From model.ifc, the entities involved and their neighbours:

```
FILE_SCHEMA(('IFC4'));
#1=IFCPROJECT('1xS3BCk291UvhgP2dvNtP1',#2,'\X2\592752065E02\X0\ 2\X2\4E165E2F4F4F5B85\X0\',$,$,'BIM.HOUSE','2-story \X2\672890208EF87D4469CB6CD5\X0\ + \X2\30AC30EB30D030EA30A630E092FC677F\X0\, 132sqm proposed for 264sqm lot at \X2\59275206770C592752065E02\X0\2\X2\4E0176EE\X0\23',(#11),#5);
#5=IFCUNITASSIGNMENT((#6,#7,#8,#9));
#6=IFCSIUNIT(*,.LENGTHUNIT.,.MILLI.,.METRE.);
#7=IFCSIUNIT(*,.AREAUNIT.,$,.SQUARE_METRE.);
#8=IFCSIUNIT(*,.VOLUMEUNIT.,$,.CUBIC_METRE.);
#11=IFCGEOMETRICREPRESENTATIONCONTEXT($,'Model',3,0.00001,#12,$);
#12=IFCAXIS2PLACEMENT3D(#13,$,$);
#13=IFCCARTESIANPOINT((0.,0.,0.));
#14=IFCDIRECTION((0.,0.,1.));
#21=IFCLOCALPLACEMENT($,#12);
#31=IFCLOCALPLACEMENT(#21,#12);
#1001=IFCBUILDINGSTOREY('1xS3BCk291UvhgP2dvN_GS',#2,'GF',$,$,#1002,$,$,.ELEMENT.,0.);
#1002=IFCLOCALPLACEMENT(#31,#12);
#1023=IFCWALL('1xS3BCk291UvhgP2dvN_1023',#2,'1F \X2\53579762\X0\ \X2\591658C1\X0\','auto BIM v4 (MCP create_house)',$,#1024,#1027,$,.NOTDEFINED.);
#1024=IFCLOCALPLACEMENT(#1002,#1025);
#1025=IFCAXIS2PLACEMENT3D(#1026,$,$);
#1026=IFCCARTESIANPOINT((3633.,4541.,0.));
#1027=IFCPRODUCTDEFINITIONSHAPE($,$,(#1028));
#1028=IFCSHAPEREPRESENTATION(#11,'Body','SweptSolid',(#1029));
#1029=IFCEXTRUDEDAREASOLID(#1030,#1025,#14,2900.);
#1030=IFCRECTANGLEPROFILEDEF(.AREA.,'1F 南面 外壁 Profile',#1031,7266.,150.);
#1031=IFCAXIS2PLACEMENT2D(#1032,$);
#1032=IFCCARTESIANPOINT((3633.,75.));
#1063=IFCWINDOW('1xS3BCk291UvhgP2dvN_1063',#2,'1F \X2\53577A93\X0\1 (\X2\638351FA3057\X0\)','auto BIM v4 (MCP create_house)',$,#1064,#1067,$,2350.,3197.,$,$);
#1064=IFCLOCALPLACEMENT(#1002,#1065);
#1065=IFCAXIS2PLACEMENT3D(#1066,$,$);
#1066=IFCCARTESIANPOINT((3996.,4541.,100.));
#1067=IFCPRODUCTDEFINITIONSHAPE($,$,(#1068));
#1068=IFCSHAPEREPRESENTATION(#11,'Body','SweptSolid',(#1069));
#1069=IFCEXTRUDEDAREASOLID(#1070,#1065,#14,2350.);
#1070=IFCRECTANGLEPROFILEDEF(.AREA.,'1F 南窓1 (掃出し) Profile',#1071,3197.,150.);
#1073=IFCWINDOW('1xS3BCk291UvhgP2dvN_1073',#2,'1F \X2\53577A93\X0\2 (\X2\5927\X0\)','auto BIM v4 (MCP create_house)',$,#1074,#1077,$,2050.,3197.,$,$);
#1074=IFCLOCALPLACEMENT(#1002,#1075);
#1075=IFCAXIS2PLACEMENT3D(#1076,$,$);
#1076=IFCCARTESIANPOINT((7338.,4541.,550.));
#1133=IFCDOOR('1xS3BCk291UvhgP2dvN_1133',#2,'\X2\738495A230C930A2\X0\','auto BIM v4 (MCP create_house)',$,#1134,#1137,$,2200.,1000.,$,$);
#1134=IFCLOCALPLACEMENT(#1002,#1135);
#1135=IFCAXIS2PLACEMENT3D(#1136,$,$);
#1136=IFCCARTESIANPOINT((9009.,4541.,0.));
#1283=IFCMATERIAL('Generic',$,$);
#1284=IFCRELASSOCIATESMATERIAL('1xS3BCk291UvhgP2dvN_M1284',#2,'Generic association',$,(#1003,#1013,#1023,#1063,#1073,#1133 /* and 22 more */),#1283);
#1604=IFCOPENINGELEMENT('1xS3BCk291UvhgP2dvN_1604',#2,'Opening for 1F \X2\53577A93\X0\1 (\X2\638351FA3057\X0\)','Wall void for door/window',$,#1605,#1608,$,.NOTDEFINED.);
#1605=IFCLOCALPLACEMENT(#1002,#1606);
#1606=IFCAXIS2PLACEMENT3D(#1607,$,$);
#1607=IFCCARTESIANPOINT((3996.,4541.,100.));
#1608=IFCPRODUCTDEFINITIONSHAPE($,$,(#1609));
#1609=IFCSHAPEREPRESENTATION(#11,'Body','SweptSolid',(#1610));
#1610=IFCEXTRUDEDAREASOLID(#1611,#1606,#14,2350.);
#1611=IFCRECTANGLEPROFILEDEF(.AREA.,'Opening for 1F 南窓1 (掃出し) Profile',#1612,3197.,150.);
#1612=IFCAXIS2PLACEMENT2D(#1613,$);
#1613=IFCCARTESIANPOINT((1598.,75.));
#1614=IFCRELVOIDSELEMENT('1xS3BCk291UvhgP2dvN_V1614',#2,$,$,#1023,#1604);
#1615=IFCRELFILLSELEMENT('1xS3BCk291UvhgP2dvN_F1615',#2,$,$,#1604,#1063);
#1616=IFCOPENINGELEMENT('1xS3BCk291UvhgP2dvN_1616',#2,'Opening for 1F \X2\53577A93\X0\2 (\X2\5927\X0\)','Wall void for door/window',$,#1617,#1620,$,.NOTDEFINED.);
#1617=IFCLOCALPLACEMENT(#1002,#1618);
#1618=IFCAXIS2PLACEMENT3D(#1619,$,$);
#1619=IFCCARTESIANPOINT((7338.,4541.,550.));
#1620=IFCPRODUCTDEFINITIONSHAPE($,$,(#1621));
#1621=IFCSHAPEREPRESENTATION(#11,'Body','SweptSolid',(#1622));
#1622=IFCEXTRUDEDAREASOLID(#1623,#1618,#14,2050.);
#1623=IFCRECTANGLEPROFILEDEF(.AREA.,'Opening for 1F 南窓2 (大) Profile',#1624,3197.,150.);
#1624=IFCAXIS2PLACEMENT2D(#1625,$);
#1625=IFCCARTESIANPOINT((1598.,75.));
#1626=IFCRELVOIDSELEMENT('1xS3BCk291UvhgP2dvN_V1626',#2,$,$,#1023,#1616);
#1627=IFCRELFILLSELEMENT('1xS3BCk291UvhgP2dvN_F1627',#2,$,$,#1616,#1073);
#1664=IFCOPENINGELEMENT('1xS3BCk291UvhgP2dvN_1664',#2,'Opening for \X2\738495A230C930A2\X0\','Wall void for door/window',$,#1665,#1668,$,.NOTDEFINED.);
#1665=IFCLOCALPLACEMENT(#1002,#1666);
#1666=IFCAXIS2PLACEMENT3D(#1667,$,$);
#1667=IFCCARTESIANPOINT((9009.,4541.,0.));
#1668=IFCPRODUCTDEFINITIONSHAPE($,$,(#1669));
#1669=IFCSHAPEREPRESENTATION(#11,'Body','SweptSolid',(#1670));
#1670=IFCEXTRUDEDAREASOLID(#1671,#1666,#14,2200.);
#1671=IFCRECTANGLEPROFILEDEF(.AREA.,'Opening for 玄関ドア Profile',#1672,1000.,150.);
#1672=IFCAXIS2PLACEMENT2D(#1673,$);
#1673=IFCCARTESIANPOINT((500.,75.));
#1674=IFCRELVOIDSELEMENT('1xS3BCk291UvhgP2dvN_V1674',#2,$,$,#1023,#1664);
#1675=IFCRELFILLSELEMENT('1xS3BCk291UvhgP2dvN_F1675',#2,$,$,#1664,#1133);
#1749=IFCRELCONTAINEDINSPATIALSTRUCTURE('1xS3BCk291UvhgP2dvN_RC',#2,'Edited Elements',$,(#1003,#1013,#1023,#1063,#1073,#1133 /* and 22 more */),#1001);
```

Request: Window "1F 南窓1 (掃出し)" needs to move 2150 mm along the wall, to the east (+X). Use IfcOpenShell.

```python
import ifcopenshell
import ifcopenshell.api.geometry
import ifcopenshell.util.placement

model = ifcopenshell.open("model.ifc")

window = model.by_guid("1xS3BCk291UvhgP2dvN_1063")
opening = window.FillsVoids[0].RelatingOpeningElement
wall = opening.VoidsElements[0].RelatingBuildingElement

wall_matrix = ifcopenshell.util.placement.get_local_placement(wall.ObjectPlacement)
shift = wall_matrix[:3, 0] * 2150.0
before = ifcopenshell.util.placement.get_local_placement(window.ObjectPlacement)[:3, 3].copy()

# The window is not placed relative to its opening, so move both.
for product in (opening, window):
    matrix = ifcopenshell.util.placement.get_local_placement(product.ObjectPlacement)
    matrix[:3, 3] += shift
    ifcopenshell.api.geometry.edit_object_placement(model, product=product, matrix=matrix, is_si=False)

after = ifcopenshell.util.placement.get_local_placement(window.ObjectPlacement)[:3, 3]
print("window moved by", (after - before).round(3) + 0.0)

model.write("model_edited.ifc")
```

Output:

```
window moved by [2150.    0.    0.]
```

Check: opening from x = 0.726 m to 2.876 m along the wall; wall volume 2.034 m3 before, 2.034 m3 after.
